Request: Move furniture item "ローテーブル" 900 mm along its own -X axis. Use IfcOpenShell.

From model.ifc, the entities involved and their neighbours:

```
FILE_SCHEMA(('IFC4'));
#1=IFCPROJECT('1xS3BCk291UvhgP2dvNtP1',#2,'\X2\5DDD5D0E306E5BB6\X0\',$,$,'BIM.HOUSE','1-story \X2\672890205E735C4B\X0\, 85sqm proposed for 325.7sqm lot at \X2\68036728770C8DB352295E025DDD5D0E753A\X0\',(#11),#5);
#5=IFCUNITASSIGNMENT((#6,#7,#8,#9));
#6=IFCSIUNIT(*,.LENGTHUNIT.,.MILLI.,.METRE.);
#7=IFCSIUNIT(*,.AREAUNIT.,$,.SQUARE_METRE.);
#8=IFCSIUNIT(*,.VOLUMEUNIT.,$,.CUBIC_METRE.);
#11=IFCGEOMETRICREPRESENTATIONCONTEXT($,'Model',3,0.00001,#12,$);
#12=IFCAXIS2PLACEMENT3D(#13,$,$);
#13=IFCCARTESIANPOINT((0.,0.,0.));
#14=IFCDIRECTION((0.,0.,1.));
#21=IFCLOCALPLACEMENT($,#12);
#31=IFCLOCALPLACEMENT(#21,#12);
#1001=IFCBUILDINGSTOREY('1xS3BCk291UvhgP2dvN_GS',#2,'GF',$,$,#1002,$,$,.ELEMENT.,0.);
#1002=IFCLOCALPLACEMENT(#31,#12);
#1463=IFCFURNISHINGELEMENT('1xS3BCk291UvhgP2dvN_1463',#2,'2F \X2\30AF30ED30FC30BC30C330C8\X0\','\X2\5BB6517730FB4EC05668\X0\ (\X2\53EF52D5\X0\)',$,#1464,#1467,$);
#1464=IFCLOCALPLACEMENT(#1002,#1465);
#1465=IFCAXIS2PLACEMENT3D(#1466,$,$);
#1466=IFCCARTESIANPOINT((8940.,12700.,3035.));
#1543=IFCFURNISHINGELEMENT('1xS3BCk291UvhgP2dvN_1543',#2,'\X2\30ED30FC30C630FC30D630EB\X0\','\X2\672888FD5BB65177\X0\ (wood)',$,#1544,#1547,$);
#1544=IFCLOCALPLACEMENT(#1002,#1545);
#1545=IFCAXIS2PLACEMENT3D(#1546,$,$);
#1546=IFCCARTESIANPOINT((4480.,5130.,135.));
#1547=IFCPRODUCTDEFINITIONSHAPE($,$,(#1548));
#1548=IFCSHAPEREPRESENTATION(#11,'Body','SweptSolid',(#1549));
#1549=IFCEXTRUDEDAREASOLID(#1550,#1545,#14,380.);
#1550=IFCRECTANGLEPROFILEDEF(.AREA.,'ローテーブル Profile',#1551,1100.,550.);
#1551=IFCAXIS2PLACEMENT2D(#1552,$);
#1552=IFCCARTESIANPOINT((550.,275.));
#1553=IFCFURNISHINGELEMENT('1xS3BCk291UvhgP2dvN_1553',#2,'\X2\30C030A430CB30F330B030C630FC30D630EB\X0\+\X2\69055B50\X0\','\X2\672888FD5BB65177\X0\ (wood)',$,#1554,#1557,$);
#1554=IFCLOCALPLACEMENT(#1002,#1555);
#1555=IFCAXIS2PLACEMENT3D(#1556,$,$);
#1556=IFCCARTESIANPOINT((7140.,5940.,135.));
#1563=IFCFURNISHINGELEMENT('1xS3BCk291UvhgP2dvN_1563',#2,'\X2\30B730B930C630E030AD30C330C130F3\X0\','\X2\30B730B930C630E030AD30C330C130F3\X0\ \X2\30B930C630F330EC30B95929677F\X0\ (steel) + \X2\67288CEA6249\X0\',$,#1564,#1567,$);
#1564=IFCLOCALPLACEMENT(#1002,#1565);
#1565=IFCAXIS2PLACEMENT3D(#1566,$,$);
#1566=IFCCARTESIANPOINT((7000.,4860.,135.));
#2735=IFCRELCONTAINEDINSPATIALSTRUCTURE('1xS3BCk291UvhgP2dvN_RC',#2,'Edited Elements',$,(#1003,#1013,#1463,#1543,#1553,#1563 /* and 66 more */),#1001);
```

```python
import ifcopenshell
import ifcopenshell.api.geometry
import ifcopenshell.util.placement
import ifcopenshell.util.unit

model = ifcopenshell.open("model.ifc")
unit_scale = ifcopenshell.util.unit.calculate_unit_scale(model)

item = model.by_guid("1xS3BCk291UvhgP2dvN_1543")
matrix = ifcopenshell.util.placement.get_local_placement(item.ObjectPlacement)
matrix[:3, 3] -= matrix[:3, 0] * 0.9 / unit_scale
ifcopenshell.api.geometry.edit_object_placement(model, product=item, matrix=matrix, is_si=False)

print(ifcopenshell.util.placement.get_local_placement(item.ObjectPlacement).round(3) + 0.0)

model.write("model_edited.ifc")
```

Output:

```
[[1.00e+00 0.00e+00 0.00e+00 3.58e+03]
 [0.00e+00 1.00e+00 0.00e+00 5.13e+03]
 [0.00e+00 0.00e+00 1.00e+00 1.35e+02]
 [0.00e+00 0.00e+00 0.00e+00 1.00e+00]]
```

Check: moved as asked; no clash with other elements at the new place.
